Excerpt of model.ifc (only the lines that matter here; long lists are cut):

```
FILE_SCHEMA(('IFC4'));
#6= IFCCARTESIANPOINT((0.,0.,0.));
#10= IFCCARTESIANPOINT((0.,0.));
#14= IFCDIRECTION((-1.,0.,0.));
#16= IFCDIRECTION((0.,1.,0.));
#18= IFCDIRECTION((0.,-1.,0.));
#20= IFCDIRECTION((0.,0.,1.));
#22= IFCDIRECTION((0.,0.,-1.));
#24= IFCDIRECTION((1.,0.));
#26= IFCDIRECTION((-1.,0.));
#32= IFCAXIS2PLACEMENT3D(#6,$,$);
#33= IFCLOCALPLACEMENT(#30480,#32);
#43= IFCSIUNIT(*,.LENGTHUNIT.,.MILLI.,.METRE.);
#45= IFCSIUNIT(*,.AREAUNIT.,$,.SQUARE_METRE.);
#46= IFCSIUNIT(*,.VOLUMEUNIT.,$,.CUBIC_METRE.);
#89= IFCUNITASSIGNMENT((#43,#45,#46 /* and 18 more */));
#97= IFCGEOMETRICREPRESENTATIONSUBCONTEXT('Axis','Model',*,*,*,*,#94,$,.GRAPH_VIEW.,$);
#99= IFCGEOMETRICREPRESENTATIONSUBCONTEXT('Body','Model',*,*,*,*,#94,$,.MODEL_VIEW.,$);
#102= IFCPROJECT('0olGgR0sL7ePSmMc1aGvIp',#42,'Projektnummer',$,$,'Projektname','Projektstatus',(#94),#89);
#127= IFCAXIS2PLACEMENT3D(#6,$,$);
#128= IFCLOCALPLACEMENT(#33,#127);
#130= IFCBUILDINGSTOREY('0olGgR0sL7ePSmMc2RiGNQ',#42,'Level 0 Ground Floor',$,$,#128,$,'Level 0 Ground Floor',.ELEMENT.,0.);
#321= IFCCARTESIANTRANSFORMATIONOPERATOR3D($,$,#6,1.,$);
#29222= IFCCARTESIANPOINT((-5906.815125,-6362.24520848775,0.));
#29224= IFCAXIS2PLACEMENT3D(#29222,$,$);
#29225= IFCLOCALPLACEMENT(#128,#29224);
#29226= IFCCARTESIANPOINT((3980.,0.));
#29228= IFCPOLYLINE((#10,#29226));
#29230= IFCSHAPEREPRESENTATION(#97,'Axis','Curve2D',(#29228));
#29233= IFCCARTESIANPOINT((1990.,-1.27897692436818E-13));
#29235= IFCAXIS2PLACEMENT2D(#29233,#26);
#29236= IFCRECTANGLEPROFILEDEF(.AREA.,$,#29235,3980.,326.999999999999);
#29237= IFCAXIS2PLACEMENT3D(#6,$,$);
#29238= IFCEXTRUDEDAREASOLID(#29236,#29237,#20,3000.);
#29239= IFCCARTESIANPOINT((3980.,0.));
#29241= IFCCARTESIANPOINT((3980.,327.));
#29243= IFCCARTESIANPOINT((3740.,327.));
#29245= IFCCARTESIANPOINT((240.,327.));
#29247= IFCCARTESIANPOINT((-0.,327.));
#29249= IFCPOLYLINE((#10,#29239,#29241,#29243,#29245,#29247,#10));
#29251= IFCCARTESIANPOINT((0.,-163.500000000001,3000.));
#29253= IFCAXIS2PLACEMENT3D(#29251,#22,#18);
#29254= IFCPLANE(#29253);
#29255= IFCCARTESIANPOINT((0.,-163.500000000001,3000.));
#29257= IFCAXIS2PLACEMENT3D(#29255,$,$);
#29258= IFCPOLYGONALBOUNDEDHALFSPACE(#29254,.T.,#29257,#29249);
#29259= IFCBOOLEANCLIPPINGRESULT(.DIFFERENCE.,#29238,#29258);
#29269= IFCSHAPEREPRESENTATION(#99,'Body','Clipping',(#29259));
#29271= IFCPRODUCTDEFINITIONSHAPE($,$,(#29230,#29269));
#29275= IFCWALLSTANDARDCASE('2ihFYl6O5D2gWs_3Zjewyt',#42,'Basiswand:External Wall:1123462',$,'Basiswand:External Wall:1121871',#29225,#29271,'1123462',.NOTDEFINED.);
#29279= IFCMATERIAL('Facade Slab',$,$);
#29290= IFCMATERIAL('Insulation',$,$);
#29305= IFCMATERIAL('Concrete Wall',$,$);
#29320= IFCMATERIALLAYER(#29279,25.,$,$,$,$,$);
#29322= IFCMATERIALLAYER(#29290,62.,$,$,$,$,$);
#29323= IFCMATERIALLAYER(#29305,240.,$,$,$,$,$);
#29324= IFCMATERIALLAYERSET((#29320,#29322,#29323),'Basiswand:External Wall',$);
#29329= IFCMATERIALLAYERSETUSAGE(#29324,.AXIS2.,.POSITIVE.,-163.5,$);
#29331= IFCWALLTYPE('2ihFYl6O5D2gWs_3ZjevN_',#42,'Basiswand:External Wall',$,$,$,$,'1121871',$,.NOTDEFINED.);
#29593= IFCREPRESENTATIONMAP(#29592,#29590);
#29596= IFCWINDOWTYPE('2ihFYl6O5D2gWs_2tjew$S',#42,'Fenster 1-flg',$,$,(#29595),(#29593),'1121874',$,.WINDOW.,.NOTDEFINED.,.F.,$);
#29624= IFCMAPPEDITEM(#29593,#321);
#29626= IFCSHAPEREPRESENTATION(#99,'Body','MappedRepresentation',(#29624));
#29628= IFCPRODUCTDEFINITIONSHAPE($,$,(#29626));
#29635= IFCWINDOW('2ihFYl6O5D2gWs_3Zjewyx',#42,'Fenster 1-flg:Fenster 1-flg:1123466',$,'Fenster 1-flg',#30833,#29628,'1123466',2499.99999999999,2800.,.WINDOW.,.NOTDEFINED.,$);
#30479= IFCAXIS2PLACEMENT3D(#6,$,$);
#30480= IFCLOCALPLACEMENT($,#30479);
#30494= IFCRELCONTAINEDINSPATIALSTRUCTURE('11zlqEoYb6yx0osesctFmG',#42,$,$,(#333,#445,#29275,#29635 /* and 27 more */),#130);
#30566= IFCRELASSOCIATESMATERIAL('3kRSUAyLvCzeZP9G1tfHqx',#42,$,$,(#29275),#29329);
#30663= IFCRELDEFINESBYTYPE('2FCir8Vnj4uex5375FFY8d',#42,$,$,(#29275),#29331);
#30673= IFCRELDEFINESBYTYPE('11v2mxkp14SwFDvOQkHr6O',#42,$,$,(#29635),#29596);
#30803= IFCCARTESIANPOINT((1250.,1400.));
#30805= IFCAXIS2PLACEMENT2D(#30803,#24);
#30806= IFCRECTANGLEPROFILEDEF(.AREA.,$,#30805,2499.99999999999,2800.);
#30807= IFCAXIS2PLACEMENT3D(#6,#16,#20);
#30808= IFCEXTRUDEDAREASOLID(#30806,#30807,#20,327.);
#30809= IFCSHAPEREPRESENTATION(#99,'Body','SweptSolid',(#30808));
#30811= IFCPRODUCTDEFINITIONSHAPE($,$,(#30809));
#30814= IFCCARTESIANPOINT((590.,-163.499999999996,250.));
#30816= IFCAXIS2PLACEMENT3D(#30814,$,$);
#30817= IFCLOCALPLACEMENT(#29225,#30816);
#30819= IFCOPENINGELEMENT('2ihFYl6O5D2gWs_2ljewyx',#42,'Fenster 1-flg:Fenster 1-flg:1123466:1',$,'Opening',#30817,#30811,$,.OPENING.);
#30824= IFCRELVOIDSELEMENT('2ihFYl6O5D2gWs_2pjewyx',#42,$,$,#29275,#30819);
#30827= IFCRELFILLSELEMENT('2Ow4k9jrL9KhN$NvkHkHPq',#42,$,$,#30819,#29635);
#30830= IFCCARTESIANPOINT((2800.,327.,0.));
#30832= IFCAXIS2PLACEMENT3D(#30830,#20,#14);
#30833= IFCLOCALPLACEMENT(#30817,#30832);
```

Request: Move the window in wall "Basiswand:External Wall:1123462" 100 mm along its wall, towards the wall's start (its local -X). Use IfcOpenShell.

```python
import ifcopenshell
import ifcopenshell.api.geometry
import ifcopenshell.util.placement

model = ifcopenshell.open("model.ifc")

window = model.by_id(29635)
opening = window.FillsVoids[0].RelatingOpeningElement
wall = opening.VoidsElements[0].RelatingBuildingElement

wall_matrix = ifcopenshell.util.placement.get_local_placement(wall.ObjectPlacement)
shift = wall_matrix[:3, 0] * -100.0
before = ifcopenshell.util.placement.get_local_placement(window.ObjectPlacement)[:3, 3].copy()

# The window is placed relative to its opening, so it follows when the opening moves.
matrix = ifcopenshell.util.placement.get_local_placement(opening.ObjectPlacement)
matrix[:3, 3] += shift
ifcopenshell.api.geometry.edit_object_placement(
    model, product=opening, matrix=matrix, is_si=False, should_transform_children=True
)

after = ifcopenshell.util.placement.get_local_placement(window.ObjectPlacement)[:3, 3]
print("window moved by", (after - before).round(3) + 0.0)

model.write("model_v2.ifc")
```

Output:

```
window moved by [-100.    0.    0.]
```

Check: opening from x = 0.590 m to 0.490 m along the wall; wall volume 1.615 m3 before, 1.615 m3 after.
